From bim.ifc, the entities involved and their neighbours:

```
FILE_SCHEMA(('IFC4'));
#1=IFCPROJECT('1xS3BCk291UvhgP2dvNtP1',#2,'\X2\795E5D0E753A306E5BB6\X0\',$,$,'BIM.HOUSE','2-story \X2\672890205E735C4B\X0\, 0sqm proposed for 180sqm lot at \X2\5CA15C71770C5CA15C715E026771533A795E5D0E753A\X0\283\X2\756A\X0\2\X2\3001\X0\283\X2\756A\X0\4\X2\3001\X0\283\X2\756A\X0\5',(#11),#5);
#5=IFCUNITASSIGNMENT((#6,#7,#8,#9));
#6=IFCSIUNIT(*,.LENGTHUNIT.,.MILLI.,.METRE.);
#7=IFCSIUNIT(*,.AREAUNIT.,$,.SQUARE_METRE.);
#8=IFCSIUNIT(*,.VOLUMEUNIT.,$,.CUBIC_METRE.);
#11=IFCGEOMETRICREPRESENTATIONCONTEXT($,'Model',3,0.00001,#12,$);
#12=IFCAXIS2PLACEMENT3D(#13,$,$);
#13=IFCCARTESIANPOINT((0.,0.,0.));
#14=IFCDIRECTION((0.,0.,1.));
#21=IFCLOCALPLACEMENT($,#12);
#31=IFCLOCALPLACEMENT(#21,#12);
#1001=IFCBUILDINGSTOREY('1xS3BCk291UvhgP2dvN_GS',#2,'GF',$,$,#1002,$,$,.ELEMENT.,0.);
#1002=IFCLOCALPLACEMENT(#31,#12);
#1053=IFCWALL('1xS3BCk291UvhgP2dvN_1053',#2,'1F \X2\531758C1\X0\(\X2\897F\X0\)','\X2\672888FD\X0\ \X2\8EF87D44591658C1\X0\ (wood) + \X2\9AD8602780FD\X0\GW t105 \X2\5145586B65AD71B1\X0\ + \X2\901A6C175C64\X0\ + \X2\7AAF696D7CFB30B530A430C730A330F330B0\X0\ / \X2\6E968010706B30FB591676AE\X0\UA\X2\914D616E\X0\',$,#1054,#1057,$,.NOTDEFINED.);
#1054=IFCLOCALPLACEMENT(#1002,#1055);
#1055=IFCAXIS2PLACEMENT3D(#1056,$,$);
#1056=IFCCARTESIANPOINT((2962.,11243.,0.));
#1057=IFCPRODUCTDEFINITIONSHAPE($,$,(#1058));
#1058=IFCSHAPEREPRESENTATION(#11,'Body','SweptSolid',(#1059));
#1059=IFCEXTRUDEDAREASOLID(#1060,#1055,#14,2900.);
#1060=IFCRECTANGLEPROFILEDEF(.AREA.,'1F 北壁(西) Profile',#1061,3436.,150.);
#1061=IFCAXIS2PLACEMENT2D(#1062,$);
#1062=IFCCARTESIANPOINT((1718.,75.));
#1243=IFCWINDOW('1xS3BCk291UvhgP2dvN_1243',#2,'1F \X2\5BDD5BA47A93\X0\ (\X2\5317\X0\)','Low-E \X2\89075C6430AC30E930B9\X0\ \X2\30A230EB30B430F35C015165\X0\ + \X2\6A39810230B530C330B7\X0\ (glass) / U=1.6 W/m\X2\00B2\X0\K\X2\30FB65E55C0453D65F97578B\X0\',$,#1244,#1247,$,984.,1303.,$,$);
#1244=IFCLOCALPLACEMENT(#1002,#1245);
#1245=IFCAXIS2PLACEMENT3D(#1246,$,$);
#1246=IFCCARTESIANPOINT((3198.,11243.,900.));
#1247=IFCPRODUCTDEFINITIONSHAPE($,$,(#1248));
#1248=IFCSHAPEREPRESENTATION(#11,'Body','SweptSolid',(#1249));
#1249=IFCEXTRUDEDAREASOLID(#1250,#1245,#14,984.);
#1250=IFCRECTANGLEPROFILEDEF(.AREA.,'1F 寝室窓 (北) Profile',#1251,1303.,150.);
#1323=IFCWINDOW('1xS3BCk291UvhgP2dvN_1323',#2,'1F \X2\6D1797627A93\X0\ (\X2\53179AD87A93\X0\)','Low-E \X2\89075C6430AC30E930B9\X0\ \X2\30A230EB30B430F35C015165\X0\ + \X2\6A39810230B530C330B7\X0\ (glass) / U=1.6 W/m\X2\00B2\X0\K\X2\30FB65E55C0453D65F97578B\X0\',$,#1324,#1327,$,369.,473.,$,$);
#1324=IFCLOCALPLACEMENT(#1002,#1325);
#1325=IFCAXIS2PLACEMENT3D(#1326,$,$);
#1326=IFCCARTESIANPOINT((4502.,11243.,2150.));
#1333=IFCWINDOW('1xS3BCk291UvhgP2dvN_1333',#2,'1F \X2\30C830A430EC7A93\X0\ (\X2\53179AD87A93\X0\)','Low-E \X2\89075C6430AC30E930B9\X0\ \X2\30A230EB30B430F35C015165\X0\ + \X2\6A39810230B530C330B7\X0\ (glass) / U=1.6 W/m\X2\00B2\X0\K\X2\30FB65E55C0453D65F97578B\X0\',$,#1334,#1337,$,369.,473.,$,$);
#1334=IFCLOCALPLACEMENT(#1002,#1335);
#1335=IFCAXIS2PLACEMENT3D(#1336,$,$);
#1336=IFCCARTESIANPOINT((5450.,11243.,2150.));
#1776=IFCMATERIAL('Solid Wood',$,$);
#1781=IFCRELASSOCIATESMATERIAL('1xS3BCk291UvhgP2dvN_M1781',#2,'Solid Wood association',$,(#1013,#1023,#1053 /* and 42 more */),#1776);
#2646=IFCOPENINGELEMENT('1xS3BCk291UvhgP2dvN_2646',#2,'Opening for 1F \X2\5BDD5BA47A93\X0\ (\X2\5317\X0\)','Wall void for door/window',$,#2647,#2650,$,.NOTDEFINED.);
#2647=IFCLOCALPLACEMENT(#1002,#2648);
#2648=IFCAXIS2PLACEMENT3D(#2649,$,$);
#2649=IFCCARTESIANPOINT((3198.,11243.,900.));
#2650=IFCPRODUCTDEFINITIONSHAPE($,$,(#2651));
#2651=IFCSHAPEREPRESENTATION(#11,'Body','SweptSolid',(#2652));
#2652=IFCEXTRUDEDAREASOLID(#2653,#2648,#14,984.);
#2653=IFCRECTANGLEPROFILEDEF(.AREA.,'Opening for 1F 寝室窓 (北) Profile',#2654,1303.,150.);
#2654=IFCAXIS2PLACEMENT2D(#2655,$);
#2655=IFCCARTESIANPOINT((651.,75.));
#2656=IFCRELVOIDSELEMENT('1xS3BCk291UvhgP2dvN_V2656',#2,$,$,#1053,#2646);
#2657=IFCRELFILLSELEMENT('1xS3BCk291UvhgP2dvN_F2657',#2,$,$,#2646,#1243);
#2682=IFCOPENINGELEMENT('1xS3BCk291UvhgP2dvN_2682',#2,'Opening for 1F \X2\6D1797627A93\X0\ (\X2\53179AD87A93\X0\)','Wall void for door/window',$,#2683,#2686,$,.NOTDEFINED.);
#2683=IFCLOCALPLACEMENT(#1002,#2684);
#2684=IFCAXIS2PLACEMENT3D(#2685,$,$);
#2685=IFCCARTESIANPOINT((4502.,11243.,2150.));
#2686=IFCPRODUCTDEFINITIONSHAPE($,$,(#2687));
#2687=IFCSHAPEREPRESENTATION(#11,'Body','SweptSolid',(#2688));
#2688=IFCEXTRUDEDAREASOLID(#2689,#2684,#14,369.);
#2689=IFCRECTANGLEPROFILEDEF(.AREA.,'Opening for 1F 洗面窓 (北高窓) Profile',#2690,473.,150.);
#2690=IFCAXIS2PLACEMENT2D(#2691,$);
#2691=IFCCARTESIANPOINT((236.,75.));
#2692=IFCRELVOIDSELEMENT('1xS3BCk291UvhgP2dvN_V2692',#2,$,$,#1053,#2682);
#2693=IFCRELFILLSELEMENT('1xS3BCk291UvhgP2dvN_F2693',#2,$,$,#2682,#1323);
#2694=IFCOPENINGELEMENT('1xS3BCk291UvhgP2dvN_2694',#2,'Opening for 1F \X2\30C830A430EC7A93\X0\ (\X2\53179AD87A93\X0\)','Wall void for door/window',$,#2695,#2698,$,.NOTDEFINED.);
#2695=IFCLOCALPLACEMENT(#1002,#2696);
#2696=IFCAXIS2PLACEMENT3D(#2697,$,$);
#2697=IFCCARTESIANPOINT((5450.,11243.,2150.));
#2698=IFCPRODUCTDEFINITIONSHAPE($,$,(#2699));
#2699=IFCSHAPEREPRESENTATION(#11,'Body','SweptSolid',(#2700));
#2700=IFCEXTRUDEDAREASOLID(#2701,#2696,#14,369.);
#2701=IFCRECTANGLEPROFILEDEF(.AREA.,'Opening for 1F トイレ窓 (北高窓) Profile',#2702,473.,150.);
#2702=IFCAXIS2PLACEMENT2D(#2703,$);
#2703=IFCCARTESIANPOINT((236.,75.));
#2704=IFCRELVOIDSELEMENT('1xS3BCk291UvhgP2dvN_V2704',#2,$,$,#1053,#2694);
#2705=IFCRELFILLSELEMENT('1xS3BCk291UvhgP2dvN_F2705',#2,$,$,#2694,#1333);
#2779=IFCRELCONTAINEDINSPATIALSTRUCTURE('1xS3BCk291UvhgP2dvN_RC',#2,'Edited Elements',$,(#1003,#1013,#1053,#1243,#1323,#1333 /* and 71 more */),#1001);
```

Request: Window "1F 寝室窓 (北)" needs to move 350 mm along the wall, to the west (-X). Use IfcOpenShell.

```python
import ifcopenshell
import ifcopenshell.api.geometry
import ifcopenshell.util.placement
import ifcopenshell.util.unit

model = ifcopenshell.open("bim.ifc")
unit_scale = ifcopenshell.util.unit.calculate_unit_scale(model)

window = model.by_id(1243)
opening = window.FillsVoids[0].RelatingOpeningElement
wall = opening.VoidsElements[0].RelatingBuildingElement

wall_matrix = ifcopenshell.util.placement.get_local_placement(wall.ObjectPlacement)
shift = wall_matrix[:3, 0] * -0.35 / unit_scale
before = ifcopenshell.util.placement.get_local_placement(window.ObjectPlacement)[:3, 3].copy()

# The window is not placed relative to its opening, so move both.
for product in (opening, window):
    matrix = ifcopenshell.util.placement.get_local_placement(product.ObjectPlacement)
    matrix[:3, 3] += shift
    ifcopenshell.api.geometry.edit_object_placement(model, product=product, matrix=matrix, is_si=False)

after = ifcopenshell.util.placement.get_local_placement(window.ObjectPlacement)[:3, 3]
print("window moved by", (after - before).round(3) + 0.0)

model.write("bim_rev.ifc")
```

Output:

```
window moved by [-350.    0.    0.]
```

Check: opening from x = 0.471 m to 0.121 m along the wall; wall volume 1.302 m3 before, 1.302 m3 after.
